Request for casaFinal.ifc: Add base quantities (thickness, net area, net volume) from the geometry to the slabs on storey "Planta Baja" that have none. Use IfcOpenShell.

First a look at what the model holds.

```python
import ifcopenshell
import ifcopenshell.util.element
import ifcopenshell.util.unit

model = ifcopenshell.open("casaFinal.ifc")
print(model.schema)
for unit_type in ("LENGTHUNIT", "AREAUNIT", "VOLUMEUNIT"):
    print(unit_type, ifcopenshell.util.unit.calculate_unit_scale(model, unit_type))
storey = next(s for s in model.by_type("IfcBuildingStorey") if s.Name == "Planta Baja")
slabs = [e for e in ifcopenshell.util.element.get_decomposition(storey) if e.is_a("IfcSlab")]
for e in sorted(slabs, key=lambda e: e.id()):
    print(e.id(), e.is_a(), e.Name, list(ifcopenshell.util.element.get_psets(e, qtos_only=True)), sep=" | ")
```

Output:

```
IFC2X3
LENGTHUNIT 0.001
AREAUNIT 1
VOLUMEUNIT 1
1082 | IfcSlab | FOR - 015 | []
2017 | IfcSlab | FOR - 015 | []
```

```python
import ifcopenshell
import ifcopenshell.api.pset
import ifcopenshell.geom
import ifcopenshell.util.element
import ifcopenshell.util.shape
import ifcopenshell.util.unit

model = ifcopenshell.open("casaFinal.ifc")
unit_scale = ifcopenshell.util.unit.calculate_unit_scale(model)
area_scale = ifcopenshell.util.unit.calculate_unit_scale(model, "AREAUNIT")
volume_scale = ifcopenshell.util.unit.calculate_unit_scale(model, "VOLUMEUNIT")
settings = ifcopenshell.geom.settings()

storey = next(s for s in model.by_type("IfcBuildingStorey") if s.Name == "Planta Baja")
slabs = [e for e in ifcopenshell.util.element.get_decomposition(storey) if e.is_a("IfcSlab")]

for e in sorted(slabs, key=lambda e: e.id()):
    if ifcopenshell.util.element.get_psets(e, qtos_only=True, should_inherit=False):
        continue
    # Geometry comes back in metres, in the element's own axes.
    shape = ifcopenshell.geom.create_shape(settings, e)
    values = {
        "Width": ifcopenshell.util.shape.get_z(shape.geometry) / unit_scale,
        "NetArea": ifcopenshell.util.shape.get_footprint_area(shape.geometry) / area_scale,
        "NetVolume": ifcopenshell.util.shape.get_volume(shape.geometry) / volume_scale,
    }
    qto = ifcopenshell.api.pset.add_qto(model, product=e, name="BaseQuantities")
    ifcopenshell.api.pset.edit_qto(model, qto=qto, properties=values)
    print(e.id(), {k: round(v, 3) for k, v in values.items()})

model.write("casaFinal_rev.ifc")
```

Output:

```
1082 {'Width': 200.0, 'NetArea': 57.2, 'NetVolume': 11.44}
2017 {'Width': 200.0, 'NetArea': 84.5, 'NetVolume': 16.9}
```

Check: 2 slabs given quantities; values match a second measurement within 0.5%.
